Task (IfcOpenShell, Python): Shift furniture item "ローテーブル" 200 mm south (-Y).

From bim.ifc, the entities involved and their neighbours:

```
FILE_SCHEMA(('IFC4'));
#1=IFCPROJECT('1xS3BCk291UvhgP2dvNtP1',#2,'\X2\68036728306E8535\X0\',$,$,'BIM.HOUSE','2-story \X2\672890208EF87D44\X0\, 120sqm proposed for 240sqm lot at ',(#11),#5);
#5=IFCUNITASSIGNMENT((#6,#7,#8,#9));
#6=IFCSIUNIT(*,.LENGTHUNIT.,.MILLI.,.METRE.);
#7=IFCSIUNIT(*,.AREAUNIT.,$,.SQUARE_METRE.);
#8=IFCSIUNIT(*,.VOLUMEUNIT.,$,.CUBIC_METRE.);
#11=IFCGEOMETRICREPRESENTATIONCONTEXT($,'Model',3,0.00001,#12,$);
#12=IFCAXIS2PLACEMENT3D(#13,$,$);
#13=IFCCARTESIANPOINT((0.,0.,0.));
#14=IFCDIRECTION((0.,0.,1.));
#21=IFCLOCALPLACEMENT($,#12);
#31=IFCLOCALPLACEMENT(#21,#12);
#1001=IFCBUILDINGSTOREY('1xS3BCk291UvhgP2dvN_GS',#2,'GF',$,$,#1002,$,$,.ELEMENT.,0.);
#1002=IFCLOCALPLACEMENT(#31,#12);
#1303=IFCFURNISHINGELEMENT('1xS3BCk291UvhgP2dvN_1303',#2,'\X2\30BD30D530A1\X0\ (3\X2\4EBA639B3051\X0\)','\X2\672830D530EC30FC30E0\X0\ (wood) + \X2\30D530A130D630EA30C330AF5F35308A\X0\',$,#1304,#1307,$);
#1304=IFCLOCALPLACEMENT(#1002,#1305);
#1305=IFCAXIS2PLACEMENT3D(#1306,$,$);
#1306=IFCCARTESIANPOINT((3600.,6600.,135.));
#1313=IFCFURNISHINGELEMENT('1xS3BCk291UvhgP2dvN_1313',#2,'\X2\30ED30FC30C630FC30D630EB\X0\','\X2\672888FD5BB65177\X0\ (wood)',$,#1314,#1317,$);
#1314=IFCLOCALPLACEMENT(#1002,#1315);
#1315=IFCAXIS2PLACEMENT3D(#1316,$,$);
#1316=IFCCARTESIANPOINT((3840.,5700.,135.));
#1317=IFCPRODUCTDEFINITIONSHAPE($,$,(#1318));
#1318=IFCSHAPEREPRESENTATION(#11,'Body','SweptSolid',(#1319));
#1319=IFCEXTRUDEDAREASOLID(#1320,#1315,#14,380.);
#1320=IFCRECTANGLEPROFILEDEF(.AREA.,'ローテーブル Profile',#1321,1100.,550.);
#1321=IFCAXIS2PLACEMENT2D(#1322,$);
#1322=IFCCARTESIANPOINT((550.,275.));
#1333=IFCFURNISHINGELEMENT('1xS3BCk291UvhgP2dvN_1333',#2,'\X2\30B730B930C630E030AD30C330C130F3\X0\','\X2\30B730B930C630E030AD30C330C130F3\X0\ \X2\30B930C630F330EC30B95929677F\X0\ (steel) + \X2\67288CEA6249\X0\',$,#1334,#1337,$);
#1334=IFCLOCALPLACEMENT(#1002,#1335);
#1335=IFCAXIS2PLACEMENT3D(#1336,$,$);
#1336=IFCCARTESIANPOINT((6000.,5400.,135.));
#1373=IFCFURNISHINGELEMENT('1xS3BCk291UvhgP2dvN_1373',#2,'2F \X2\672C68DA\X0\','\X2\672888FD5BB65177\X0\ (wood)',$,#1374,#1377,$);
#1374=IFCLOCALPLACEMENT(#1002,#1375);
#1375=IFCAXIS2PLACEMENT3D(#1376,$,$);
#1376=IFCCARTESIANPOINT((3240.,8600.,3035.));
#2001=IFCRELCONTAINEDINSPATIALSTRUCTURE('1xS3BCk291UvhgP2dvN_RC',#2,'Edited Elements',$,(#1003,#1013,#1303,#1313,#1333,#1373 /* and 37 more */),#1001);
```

```python
import ifcopenshell
import ifcopenshell.api.geometry
import ifcopenshell.util.placement

model = ifcopenshell.open("bim.ifc")

item = model.by_guid("1xS3BCk291UvhgP2dvN_1313")
matrix = ifcopenshell.util.placement.get_local_placement(item.ObjectPlacement)
matrix[1, 3] -= 200.0
ifcopenshell.api.geometry.edit_object_placement(model, product=item, matrix=matrix, is_si=False)

print(ifcopenshell.util.placement.get_local_placement(item.ObjectPlacement).round(3) + 0.0)

model.write("bim_updated.ifc")
```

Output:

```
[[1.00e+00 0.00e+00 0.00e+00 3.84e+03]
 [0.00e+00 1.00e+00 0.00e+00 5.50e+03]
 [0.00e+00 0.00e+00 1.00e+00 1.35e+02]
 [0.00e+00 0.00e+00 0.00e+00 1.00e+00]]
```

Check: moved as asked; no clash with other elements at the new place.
